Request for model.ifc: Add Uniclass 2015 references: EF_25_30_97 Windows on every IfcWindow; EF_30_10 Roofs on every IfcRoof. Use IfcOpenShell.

First a look at what the model holds.

```python
import ifcopenshell

model = ifcopenshell.open("model.ifc")
print(model.schema)
print("classifications:", [c.Name for c in model.by_type("IfcClassification")])
for ifc_class in ("IfcDoor", "IfcRoof", "IfcStair", "IfcWall", "IfcWindow"):
    print(ifc_class, len(model.by_type(ifc_class)))
```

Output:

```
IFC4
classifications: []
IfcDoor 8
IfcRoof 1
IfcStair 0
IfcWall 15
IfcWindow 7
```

```python
import ifcopenshell
import ifcopenshell.api.classification

model = ifcopenshell.open("model.ifc")

system = ifcopenshell.api.classification.add_classification(model, classification="Uniclass 2015")

codes = {
    "IfcWindow": ("EF_25_30_97", "Windows"),
    "IfcRoof": ("EF_30_10", "Roofs"),
}
for ifc_class, (code, name) in codes.items():
    products = model.by_type(ifc_class)
    ifcopenshell.api.classification.add_reference(
        model, products=products, classification=system, identification=code, name=name
    )
    print(code, len(products))

model.write("model_edited.ifc")
```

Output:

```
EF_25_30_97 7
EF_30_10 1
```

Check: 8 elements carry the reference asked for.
